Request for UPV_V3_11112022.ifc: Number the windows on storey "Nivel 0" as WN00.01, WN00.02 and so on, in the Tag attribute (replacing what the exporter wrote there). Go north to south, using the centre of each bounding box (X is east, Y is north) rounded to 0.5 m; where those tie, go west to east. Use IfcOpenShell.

First a look at what the model holds.

```python
import ifcopenshell
import ifcopenshell.util.element
import ifcopenshell.util.placement

model = ifcopenshell.open("UPV_V3_11112022.ifc")
print(model.schema)
storey = next(s for s in model.by_type("IfcBuildingStorey") if s.Name == "Nivel 0")
windows = [e for e in ifcopenshell.util.element.get_decomposition(storey) if e.is_a("IfcWindow")]
for e in sorted(windows, key=lambda e: e.id()):
    origin = ifcopenshell.util.placement.get_local_placement(e.ObjectPlacement)[:3, 3]
    print(e.id(), e.Tag, e.Name, origin.round(2) + 0.0, sep=" | ")
```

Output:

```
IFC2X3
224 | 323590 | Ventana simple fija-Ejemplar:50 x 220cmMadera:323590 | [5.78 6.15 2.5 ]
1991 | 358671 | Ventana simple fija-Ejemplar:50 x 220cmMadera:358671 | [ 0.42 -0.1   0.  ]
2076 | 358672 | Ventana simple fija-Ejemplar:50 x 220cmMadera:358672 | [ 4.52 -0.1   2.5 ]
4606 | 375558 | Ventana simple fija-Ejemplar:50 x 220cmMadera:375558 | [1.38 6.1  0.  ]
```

```python
import ifcopenshell
import ifcopenshell.geom
import ifcopenshell.util.element
import ifcopenshell.util.shape

model = ifcopenshell.open("UPV_V3_11112022.ifc")
settings = ifcopenshell.geom.settings()
settings.set("use-world-coords", True)


def centre(element):
    shape = ifcopenshell.geom.create_shape(settings, element)
    return ifcopenshell.util.shape.get_bbox_centroid(shape.geometry)


storey = next(s for s in model.by_type("IfcBuildingStorey") if s.Name == "Nivel 0")
windows = [e for e in ifcopenshell.util.element.get_decomposition(storey) if e.is_a("IfcWindow")]

# Insertion points can sit at a corner or the storey origin, so sort by the geometry (in metres).
centres = {e: centre(e) for e in windows}
windows.sort(key=lambda e: (-round(centres[e][1] / 0.5), centres[e][0]))

for i, e in enumerate(windows, start=1):
    number = f"WN00.{i:02d}"
    e.Tag = number
    print(e.id(), number)

model.write("UPV_V3_11112022_updated.ifc")
```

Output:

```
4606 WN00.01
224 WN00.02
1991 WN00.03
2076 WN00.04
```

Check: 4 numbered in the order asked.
